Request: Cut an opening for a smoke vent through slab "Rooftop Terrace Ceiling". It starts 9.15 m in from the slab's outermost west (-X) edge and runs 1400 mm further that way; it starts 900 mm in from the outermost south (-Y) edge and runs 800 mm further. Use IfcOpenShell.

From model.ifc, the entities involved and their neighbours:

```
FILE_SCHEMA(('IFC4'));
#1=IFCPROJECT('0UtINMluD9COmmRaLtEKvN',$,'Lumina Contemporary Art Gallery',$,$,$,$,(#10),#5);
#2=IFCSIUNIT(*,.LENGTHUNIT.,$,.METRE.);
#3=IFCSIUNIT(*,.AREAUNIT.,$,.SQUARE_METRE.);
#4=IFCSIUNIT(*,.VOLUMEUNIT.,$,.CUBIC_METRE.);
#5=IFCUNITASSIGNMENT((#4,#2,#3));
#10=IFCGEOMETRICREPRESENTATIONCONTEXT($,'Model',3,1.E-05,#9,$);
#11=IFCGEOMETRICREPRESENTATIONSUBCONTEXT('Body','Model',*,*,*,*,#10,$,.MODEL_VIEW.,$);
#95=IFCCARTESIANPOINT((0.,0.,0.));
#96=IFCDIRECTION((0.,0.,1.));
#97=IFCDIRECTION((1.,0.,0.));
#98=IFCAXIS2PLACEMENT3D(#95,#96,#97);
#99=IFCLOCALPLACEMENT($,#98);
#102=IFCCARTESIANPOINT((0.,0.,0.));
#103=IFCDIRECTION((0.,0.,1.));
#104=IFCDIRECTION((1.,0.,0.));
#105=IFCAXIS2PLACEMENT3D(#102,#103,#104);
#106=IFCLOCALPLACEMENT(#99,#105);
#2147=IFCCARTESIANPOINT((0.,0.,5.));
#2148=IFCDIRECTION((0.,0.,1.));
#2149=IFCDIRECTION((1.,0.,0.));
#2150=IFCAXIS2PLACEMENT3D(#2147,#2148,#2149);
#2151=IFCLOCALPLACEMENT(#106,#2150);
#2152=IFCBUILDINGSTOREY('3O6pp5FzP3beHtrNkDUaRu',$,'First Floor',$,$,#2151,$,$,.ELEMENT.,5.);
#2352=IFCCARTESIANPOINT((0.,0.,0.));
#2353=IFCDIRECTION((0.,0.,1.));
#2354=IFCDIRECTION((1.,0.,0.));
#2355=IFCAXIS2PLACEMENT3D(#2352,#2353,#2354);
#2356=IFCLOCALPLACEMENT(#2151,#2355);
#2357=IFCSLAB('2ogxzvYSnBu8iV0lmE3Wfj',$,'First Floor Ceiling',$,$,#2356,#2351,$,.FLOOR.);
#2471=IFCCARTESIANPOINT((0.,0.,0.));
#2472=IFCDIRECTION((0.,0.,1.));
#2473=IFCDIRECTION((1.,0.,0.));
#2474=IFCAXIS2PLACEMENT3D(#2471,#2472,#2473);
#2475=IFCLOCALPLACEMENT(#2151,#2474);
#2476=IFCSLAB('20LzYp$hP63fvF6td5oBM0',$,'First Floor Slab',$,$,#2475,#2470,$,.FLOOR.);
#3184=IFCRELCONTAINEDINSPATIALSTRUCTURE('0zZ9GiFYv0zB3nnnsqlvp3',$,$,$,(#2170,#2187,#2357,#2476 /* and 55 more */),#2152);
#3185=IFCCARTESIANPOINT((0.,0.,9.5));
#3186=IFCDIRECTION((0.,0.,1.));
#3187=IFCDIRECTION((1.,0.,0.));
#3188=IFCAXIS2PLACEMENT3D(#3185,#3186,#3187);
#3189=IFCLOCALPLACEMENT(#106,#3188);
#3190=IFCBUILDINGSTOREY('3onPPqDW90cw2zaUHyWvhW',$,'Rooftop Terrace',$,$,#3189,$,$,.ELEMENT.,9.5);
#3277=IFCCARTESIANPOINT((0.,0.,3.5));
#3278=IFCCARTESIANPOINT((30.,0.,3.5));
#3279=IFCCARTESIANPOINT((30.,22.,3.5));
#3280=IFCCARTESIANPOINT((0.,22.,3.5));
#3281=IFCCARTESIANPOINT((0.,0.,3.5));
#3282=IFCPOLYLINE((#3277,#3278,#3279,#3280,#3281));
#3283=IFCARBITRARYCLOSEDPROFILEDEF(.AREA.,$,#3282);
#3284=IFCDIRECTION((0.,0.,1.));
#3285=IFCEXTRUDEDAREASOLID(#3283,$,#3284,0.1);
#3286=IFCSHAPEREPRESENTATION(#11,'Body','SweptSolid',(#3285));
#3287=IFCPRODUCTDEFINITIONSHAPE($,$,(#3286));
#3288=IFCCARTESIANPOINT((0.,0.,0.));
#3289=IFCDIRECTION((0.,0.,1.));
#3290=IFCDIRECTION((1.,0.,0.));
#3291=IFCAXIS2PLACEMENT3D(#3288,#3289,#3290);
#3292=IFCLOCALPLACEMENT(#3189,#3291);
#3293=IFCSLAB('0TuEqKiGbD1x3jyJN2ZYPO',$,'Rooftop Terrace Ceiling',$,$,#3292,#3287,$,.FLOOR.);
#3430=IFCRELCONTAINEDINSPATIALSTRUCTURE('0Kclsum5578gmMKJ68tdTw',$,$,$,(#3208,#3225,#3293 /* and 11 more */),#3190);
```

```python
import numpy as np
import ifcopenshell
import ifcopenshell.api.feature
import ifcopenshell.api.geometry
import ifcopenshell.api.root
import ifcopenshell.geom
import ifcopenshell.util.placement
import ifcopenshell.util.representation
import ifcopenshell.util.shape
import ifcopenshell.util.unit

model = ifcopenshell.open("model.ifc")
unit_scale = ifcopenshell.util.unit.calculate_unit_scale(model)
settings = ifcopenshell.geom.settings()


def volume(element):
    """Net volume in cubic metres, openings subtracted."""
    shape = ifcopenshell.geom.create_shape(settings, element)
    return ifcopenshell.util.shape.get_volume(shape.geometry)


slab = model.by_guid("0TuEqKiGbD1x3jyJN2ZYPO")
before = volume(slab)

# Extent in the slab's own axes, in metres. The edges named are its -X and -Y sides.
slab_shape = ifcopenshell.geom.create_shape(settings, slab)
vertices = ifcopenshell.util.shape.get_vertices(slab_shape.geometry)
x_min, y_min, bottom = vertices.min(axis=0)
top = vertices[:, 2].max()

opening = ifcopenshell.api.root.create_entity(model, ifc_class="IfcOpeningElement", name="Smoke vent opening", predefined_type="OPENING")
context = ifcopenshell.util.representation.get_context(model, "Model", "Body", "MODEL_VIEW")
width, depth = 1.4, 0.8
outline = [(0.0, 0.0), (width, 0.0), (width, depth), (0.0, depth), (0.0, 0.0)]
# Overshoot both faces by 50 mm so the cut is clean.
shape = ifcopenshell.api.geometry.add_slab_representation(
    model, context=context, depth=top - bottom + 0.1, polyline=outline
)
ifcopenshell.api.geometry.assign_representation(model, product=opening, representation=shape)

matrix = ifcopenshell.util.placement.get_local_placement(slab.ObjectPlacement)
matrix[:, 3] = matrix @ np.append(np.array([x_min + 9.15, y_min + 0.9, bottom - 0.05]) / unit_scale, 1.0)
ifcopenshell.api.geometry.edit_object_placement(model, product=opening, matrix=matrix, is_si=False)
ifcopenshell.api.feature.add_feature(model, feature=opening, element=slab)

after = volume(slab)

print(f"slab volume {before:.3f} -> {after:.3f} m3")

model.write("model-out.ifc")
```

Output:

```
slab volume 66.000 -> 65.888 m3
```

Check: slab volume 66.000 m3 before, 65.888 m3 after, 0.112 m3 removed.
